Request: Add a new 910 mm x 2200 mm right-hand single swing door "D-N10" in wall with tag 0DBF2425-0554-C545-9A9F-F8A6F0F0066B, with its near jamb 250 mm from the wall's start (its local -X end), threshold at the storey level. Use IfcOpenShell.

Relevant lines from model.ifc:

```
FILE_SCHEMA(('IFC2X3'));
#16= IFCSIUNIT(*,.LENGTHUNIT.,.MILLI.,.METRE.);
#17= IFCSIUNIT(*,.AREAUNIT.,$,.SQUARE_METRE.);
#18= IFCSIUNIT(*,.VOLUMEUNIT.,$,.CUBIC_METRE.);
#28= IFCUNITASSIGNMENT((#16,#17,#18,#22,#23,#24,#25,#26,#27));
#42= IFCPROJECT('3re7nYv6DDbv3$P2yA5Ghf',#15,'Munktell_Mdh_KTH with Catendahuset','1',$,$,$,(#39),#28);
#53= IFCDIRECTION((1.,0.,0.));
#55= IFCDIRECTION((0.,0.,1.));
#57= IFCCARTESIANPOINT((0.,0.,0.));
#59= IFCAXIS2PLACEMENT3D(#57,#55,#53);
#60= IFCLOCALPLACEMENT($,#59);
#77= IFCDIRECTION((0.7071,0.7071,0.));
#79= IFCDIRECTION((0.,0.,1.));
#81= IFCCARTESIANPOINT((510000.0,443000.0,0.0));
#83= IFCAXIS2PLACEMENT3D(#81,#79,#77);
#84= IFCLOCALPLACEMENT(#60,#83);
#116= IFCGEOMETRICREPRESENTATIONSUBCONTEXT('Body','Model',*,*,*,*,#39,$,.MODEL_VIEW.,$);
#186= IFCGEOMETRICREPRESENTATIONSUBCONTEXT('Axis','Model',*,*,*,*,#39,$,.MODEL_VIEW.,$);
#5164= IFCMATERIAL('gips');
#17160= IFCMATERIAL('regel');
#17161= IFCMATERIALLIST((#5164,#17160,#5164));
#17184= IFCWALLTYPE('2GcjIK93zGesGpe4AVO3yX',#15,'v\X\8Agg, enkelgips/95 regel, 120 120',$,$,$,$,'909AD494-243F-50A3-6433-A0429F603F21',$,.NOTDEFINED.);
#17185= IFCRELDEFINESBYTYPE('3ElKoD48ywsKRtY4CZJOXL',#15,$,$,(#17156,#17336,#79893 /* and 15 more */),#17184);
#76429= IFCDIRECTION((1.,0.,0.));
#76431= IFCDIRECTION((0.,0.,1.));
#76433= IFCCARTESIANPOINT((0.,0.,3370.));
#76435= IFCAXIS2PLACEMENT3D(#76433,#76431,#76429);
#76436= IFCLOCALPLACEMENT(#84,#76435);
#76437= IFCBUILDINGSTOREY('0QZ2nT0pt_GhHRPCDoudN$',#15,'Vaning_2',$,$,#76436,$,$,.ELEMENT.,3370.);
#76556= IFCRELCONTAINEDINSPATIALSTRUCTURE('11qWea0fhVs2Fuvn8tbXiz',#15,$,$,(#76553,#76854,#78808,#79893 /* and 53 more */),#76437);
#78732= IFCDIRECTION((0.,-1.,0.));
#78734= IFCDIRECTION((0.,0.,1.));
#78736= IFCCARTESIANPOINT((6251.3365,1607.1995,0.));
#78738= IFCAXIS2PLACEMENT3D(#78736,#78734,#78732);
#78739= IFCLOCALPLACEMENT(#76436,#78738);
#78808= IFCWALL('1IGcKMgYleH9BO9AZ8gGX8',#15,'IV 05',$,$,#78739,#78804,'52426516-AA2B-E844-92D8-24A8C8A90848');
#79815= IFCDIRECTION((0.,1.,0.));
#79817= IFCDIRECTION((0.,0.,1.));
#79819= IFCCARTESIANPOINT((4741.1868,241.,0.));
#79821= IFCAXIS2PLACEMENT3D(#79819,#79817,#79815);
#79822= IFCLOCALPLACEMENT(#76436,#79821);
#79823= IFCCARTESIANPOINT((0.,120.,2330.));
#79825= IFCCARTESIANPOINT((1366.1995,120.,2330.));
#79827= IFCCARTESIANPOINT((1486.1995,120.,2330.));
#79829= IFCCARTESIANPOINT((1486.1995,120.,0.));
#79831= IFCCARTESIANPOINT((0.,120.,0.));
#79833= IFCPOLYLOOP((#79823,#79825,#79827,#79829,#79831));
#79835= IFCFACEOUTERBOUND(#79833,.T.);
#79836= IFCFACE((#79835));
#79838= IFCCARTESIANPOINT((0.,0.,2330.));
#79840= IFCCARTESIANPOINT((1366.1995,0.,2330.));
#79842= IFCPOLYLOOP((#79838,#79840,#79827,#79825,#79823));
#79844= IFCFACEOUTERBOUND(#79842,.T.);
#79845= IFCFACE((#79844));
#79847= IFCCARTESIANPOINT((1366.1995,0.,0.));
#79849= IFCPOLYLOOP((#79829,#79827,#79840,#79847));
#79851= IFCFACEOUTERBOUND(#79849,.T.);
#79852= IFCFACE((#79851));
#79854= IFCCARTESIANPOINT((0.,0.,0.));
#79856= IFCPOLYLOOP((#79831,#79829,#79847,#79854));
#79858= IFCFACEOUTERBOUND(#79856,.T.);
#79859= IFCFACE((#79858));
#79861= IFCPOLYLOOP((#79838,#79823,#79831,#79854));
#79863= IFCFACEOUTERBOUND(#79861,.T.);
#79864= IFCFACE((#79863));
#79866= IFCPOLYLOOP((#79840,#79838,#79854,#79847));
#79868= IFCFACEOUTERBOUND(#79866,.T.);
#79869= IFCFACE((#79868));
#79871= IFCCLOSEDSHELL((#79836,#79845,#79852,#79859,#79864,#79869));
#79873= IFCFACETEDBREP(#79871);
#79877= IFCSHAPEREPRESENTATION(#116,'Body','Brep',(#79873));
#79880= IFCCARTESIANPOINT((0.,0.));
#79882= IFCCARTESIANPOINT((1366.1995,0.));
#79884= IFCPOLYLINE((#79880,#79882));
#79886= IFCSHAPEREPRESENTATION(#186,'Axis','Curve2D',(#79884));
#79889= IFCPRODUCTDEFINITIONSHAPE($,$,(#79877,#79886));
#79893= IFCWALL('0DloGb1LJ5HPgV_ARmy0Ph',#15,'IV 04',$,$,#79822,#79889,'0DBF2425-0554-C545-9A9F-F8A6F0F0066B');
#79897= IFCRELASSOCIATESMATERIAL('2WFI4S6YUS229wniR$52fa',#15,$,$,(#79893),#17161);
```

```python
import numpy as np
import ifcopenshell
import ifcopenshell.api.feature
import ifcopenshell.api.geometry
import ifcopenshell.api.root
import ifcopenshell.api.spatial
import ifcopenshell.api.type
import ifcopenshell.geom
import ifcopenshell.util.element
import ifcopenshell.util.placement
import ifcopenshell.util.representation
import ifcopenshell.util.shape
import ifcopenshell.util.unit

model = ifcopenshell.open("model.ifc")
unit_scale = ifcopenshell.util.unit.calculate_unit_scale(model)
settings = ifcopenshell.geom.settings()


def volume(element):
    """Net volume in cubic metres, openings subtracted."""
    shape = ifcopenshell.geom.create_shape(settings, element)
    return ifcopenshell.util.shape.get_volume(shape.geometry)


wall = model.by_id(79893)
storey = ifcopenshell.util.element.get_container(wall, ifc_class="IfcBuildingStorey")
context = ifcopenshell.util.representation.get_context(model, "Model", "Body", "MODEL_VIEW")
before = volume(wall)

width, height, from_end, sill = 0.91, 2.2, 0.25, 0.0  # metres

# The wall runs along its own X axis, and the end named is its -X end.
wall_shape = ifcopenshell.geom.create_shape(settings, wall)
x, y, z = ifcopenshell.util.shape.get_vertices(wall_shape.geometry).T
start = x.min() + from_end
face, thickness = float(y.min()), float(y.max() - y.min())
wall_matrix = ifcopenshell.util.placement.get_local_placement(wall.ObjectPlacement)
level = ifcopenshell.util.placement.get_local_placement(storey.ObjectPlacement)[2, 3]


def in_wall(x, y):
    """Placement at x, y metres in the wall's axes, at sill height."""
    matrix = wall_matrix.copy()
    matrix[:, 3] = wall_matrix @ np.array([x / unit_scale, y / unit_scale, 0.0, 1.0])
    matrix[2, 3] = level + sill / unit_scale
    return matrix


# Opening: a box that overshoots both wall faces by 50 mm.
opening = ifcopenshell.api.root.create_entity(model, ifc_class="IfcOpeningElement")
box = ifcopenshell.api.geometry.add_wall_representation(
    model, context=context, length=width, height=height, thickness=thickness + 0.1
)
ifcopenshell.api.geometry.assign_representation(model, product=opening, representation=box)
ifcopenshell.api.geometry.edit_object_placement(model, product=opening, matrix=in_wall(start, face - 0.05), is_si=False)
ifcopenshell.api.feature.add_feature(model, feature=opening, element=wall)

door = ifcopenshell.api.root.create_entity(model, ifc_class="IfcDoor", name="D-N10")
door.OverallWidth, door.OverallHeight = width / unit_scale, height / unit_scale
body = ifcopenshell.api.geometry.add_door_representation(
    model,
    context=context,
    overall_width=door.OverallWidth,
    overall_height=door.OverallHeight,
    operation_type="SINGLE_SWING_RIGHT",
    lining_properties={"LiningDepth": thickness / unit_scale, "ThresholdDepth": thickness / unit_scale},
)
ifcopenshell.api.geometry.assign_representation(model, product=door, representation=body)
ifcopenshell.api.spatial.assign_container(model, products=[door], relating_structure=storey)
fills = ifcopenshell.api.feature.add_filling(model, opening=opening, element=door)
fills.OwnerHistory = door.OwnerHistory  # required in IFC2X3

# IFC2X3 keeps the operation on the door style.
style = ifcopenshell.api.root.create_entity(model, ifc_class="IfcDoorStyle", name="D-N10")
style.OperationType, style.ConstructionType = "SINGLE_SWING_RIGHT", "NOTDEFINED"
style.ParameterTakesPrecedence = style.Sizeable = False
ifcopenshell.api.type.assign_type(model, related_objects=[door], relating_type=style)

# The lining spans the wall, so the door starts at the wall face.
ifcopenshell.api.geometry.edit_object_placement(model, product=door, matrix=in_wall(start, face), is_si=False)

after = volume(wall)

print(f"wall volume {before:.3f} -> {after:.3f} m3")

model.write("model_rev.ifc")
```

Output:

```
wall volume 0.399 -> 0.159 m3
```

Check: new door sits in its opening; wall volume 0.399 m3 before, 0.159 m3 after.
